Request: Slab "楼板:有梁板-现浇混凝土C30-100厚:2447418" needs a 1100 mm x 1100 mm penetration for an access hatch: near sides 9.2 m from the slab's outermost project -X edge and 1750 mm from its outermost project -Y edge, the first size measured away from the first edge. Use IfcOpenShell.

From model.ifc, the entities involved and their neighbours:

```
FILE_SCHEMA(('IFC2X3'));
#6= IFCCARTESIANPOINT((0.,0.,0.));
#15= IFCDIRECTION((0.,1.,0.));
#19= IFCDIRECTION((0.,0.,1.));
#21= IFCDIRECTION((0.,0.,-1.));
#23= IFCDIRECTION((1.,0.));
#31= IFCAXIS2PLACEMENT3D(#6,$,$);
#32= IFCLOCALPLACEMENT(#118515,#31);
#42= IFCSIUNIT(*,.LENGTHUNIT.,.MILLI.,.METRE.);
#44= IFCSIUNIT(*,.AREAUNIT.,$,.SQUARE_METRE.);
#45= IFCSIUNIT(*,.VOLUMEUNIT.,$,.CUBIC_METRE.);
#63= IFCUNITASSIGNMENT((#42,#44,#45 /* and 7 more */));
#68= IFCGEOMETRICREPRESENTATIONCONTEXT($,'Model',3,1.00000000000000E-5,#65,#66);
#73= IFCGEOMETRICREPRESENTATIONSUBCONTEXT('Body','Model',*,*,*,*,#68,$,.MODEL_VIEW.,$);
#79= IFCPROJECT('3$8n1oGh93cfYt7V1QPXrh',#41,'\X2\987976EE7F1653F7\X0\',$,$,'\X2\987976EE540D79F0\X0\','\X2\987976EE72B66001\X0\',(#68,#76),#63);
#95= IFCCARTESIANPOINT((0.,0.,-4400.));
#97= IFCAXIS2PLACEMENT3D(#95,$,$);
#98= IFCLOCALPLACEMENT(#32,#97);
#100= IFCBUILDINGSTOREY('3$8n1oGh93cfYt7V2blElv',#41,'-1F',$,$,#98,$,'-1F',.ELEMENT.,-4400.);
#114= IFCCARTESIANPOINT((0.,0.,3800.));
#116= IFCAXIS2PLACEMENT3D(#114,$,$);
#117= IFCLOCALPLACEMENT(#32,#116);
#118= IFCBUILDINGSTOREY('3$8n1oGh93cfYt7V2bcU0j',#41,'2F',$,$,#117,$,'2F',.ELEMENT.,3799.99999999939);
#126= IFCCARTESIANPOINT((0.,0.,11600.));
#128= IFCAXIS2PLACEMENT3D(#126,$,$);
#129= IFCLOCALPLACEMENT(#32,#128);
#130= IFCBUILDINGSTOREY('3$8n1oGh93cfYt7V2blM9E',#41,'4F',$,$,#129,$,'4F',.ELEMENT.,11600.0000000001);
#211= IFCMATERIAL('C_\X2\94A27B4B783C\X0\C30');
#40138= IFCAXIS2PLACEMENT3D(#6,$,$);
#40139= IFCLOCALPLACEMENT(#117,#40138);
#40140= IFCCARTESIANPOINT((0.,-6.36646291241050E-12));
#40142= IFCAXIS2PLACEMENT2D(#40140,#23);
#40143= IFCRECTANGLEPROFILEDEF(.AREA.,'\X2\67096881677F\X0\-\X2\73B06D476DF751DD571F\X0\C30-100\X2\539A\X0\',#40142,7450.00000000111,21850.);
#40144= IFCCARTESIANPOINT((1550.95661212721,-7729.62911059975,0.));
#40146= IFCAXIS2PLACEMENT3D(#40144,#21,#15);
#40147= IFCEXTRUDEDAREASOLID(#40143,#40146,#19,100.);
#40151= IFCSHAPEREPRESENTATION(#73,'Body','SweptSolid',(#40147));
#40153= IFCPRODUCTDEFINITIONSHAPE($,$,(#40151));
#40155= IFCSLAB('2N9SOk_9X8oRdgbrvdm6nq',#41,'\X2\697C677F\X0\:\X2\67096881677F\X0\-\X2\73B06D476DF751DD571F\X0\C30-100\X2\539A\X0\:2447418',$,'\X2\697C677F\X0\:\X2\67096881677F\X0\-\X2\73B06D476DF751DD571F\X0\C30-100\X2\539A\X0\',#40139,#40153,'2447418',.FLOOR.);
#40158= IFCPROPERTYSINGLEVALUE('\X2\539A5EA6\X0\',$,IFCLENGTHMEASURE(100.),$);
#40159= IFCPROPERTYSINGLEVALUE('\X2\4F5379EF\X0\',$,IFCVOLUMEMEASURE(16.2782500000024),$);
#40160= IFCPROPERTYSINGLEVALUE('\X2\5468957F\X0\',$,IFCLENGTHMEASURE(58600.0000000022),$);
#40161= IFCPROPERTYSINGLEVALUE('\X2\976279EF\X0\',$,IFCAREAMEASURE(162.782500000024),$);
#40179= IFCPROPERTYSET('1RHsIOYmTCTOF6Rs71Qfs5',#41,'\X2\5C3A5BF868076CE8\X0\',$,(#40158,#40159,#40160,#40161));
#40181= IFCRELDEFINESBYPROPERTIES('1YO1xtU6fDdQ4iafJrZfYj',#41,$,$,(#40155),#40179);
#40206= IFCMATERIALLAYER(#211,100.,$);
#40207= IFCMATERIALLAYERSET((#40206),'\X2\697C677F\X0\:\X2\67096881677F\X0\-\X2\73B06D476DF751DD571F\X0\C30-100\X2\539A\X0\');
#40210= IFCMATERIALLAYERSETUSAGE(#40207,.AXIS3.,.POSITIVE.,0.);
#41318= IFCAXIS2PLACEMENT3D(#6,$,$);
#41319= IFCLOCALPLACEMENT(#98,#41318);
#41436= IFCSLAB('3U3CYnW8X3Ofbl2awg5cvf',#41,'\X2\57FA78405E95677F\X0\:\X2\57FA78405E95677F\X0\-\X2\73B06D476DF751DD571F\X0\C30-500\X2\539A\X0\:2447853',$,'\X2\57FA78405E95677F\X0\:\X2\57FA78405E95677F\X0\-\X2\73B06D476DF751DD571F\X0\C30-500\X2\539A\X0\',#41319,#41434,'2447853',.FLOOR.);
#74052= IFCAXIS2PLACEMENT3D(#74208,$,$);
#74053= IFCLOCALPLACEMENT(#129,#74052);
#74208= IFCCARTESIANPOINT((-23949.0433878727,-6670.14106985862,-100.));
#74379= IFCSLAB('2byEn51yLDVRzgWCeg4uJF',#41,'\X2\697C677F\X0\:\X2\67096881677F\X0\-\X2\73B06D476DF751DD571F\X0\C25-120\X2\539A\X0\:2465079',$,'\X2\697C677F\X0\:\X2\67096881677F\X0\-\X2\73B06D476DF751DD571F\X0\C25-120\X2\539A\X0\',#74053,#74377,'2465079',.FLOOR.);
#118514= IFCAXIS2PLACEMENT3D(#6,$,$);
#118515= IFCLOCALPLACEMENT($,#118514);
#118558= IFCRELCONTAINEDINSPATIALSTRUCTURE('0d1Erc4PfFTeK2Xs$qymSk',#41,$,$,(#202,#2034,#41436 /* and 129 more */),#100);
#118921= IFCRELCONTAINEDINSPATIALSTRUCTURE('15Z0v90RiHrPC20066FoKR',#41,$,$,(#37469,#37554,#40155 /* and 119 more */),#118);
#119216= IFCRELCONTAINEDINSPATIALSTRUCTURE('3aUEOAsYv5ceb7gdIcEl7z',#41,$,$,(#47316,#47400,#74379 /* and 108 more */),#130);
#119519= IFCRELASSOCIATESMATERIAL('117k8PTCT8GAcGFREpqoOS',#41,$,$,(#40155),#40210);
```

```python
import numpy as np
import ifcopenshell
import ifcopenshell.api.feature
import ifcopenshell.api.geometry
import ifcopenshell.api.pset
import ifcopenshell.api.root
import ifcopenshell.geom
import ifcopenshell.util.element
import ifcopenshell.util.placement
import ifcopenshell.util.representation
import ifcopenshell.util.shape
import ifcopenshell.util.unit

model = ifcopenshell.open("model.ifc")
unit_scale = ifcopenshell.util.unit.calculate_unit_scale(model)
area_scale = ifcopenshell.util.unit.calculate_unit_scale(model, "AREAUNIT")
volume_scale = ifcopenshell.util.unit.calculate_unit_scale(model, "VOLUMEUNIT")
settings = ifcopenshell.geom.settings()


def volume(element):
    """Net volume in cubic metres, openings subtracted."""
    shape = ifcopenshell.geom.create_shape(settings, element)
    return ifcopenshell.util.shape.get_volume(shape.geometry)


slab = model.by_id(40155)
before = volume(slab)

# Extent in the slab's own axes, in metres. The edges named are its -X and -Y sides.
slab_shape = ifcopenshell.geom.create_shape(settings, slab)
vertices = ifcopenshell.util.shape.get_vertices(slab_shape.geometry)
x_min, y_min, bottom = vertices.min(axis=0)
top = vertices[:, 2].max()

opening = ifcopenshell.api.root.create_entity(model, ifc_class="IfcOpeningElement", name="Access hatch opening")
context = ifcopenshell.util.representation.get_context(model, "Model", "Body", "MODEL_VIEW")
width, depth = 1.1, 1.1
outline = [(0.0, 0.0), (width, 0.0), (width, depth), (0.0, depth), (0.0, 0.0)]
# Overshoot both faces by 50 mm so the cut is clean.
shape = ifcopenshell.api.geometry.add_slab_representation(
    model, context=context, depth=top - bottom + 0.1, polyline=outline
)
ifcopenshell.api.geometry.assign_representation(model, product=opening, representation=shape)

matrix = ifcopenshell.util.placement.get_local_placement(slab.ObjectPlacement)
matrix[:, 3] = matrix @ np.append(np.array([x_min + 9.2, y_min + 1.75, bottom - 0.05]) / unit_scale, 1.0)
ifcopenshell.api.geometry.edit_object_placement(model, product=opening, matrix=matrix, is_si=False)
ifcopenshell.api.feature.add_feature(model, feature=opening, element=slab)

after = volume(slab)

# Update the slab's stored quantities.
pset = model.by_id(ifcopenshell.util.element.get_pset(slab, "尺寸标注", should_inherit=False)["id"])
ifcopenshell.api.pset.edit_pset(model, pset=pset, properties={
    "体积": model.create_entity("IfcVolumeMeasure", after / volume_scale),
    "面积": model.create_entity("IfcAreaMeasure", after / (top - bottom) / area_scale),
})

print(f"slab volume {before:.3f} -> {after:.3f} m3")

model.write("model_rev.ifc")
```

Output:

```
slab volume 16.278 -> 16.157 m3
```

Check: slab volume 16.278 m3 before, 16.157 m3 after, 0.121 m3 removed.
